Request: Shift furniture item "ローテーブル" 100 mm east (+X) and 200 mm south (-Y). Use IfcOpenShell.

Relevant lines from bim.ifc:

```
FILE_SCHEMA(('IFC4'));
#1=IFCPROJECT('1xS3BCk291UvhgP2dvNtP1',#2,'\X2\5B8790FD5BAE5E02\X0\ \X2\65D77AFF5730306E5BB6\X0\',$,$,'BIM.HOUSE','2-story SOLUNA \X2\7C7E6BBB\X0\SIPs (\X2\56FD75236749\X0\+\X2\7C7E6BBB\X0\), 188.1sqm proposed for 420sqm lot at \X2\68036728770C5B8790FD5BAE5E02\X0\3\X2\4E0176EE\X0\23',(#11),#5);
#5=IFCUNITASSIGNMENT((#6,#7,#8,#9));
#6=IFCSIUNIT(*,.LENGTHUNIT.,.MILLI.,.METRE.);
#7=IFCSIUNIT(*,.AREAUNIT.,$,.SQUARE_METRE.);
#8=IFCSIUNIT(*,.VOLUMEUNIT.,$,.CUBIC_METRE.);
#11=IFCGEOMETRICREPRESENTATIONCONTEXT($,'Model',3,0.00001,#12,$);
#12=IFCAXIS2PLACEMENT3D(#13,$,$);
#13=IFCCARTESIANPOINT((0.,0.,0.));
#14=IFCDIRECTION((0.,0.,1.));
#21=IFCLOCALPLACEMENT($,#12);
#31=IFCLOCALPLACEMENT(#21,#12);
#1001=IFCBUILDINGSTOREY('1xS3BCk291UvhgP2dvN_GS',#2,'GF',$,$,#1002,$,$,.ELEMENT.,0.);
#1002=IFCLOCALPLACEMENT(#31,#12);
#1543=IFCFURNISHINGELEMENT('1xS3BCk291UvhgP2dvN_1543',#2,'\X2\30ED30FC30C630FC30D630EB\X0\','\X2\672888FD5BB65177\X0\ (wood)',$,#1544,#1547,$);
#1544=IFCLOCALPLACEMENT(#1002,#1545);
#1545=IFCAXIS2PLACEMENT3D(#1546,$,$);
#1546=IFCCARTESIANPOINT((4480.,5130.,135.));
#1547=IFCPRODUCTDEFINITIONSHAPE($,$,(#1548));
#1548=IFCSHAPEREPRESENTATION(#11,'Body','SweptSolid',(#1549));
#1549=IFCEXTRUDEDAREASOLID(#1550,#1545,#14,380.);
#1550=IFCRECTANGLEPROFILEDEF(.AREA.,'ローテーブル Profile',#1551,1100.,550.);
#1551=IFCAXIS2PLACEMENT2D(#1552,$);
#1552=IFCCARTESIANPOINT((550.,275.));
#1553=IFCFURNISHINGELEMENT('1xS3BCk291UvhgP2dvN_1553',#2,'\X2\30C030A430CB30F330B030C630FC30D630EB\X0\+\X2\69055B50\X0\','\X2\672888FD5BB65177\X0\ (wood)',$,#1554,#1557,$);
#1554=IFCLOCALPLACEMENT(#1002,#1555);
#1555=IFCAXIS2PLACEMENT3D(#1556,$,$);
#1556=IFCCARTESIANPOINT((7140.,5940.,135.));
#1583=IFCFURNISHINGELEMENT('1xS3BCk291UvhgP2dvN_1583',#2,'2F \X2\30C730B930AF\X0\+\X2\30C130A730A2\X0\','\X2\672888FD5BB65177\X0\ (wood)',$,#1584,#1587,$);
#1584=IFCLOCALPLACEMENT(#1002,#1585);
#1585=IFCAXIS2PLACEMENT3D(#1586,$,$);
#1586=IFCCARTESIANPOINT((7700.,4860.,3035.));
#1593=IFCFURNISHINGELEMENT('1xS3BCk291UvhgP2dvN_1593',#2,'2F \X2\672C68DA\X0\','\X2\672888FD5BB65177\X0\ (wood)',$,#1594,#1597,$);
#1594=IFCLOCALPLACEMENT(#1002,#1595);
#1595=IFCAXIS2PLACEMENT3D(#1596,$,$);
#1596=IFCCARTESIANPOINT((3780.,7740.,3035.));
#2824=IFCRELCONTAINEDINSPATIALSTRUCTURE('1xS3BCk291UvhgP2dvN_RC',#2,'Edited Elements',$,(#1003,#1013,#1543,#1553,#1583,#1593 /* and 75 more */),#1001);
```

```python
import ifcopenshell
import ifcopenshell.api.geometry
import ifcopenshell.util.placement
import ifcopenshell.util.unit

model = ifcopenshell.open("bim.ifc")
unit_scale = ifcopenshell.util.unit.calculate_unit_scale(model)

item = model.by_guid("1xS3BCk291UvhgP2dvN_1543")
matrix = ifcopenshell.util.placement.get_local_placement(item.ObjectPlacement)
matrix[0, 3] += 0.1 / unit_scale
matrix[1, 3] -= 0.2 / unit_scale
ifcopenshell.api.geometry.edit_object_placement(model, product=item, matrix=matrix, is_si=False)

print(ifcopenshell.util.placement.get_local_placement(item.ObjectPlacement).round(3) + 0.0)

model.write("bim_edited.ifc")
```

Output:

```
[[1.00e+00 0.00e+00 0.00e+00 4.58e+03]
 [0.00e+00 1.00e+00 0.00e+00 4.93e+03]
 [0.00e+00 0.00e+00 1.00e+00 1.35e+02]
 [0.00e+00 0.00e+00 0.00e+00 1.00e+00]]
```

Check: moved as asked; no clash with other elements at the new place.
